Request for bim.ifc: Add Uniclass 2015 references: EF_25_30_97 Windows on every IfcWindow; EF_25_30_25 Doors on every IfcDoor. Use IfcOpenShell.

First a look at what the model holds.

```python
import ifcopenshell

model = ifcopenshell.open("bim.ifc")
print(model.schema)
print("classifications:", [c.Name for c in model.by_type("IfcClassification")])
for ifc_class in ("IfcDoor", "IfcRoof", "IfcStair", "IfcWall", "IfcWindow"):
    print(ifc_class, len(model.by_type(ifc_class)))
```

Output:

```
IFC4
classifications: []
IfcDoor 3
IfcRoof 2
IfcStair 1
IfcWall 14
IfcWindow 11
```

```python
import ifcopenshell
import ifcopenshell.api.classification

model = ifcopenshell.open("bim.ifc")

system = ifcopenshell.api.classification.add_classification(model, classification="Uniclass 2015")

codes = {
    "IfcWindow": ("EF_25_30_97", "Windows"),
    "IfcDoor": ("EF_25_30_25", "Doors"),
}
for ifc_class, (code, name) in codes.items():
    products = model.by_type(ifc_class)
    ifcopenshell.api.classification.add_reference(
        model, products=products, classification=system, identification=code, name=name
    )
    print(code, len(products))

model.write("bim-out.ifc")
```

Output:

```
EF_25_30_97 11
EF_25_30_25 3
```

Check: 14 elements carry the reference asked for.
